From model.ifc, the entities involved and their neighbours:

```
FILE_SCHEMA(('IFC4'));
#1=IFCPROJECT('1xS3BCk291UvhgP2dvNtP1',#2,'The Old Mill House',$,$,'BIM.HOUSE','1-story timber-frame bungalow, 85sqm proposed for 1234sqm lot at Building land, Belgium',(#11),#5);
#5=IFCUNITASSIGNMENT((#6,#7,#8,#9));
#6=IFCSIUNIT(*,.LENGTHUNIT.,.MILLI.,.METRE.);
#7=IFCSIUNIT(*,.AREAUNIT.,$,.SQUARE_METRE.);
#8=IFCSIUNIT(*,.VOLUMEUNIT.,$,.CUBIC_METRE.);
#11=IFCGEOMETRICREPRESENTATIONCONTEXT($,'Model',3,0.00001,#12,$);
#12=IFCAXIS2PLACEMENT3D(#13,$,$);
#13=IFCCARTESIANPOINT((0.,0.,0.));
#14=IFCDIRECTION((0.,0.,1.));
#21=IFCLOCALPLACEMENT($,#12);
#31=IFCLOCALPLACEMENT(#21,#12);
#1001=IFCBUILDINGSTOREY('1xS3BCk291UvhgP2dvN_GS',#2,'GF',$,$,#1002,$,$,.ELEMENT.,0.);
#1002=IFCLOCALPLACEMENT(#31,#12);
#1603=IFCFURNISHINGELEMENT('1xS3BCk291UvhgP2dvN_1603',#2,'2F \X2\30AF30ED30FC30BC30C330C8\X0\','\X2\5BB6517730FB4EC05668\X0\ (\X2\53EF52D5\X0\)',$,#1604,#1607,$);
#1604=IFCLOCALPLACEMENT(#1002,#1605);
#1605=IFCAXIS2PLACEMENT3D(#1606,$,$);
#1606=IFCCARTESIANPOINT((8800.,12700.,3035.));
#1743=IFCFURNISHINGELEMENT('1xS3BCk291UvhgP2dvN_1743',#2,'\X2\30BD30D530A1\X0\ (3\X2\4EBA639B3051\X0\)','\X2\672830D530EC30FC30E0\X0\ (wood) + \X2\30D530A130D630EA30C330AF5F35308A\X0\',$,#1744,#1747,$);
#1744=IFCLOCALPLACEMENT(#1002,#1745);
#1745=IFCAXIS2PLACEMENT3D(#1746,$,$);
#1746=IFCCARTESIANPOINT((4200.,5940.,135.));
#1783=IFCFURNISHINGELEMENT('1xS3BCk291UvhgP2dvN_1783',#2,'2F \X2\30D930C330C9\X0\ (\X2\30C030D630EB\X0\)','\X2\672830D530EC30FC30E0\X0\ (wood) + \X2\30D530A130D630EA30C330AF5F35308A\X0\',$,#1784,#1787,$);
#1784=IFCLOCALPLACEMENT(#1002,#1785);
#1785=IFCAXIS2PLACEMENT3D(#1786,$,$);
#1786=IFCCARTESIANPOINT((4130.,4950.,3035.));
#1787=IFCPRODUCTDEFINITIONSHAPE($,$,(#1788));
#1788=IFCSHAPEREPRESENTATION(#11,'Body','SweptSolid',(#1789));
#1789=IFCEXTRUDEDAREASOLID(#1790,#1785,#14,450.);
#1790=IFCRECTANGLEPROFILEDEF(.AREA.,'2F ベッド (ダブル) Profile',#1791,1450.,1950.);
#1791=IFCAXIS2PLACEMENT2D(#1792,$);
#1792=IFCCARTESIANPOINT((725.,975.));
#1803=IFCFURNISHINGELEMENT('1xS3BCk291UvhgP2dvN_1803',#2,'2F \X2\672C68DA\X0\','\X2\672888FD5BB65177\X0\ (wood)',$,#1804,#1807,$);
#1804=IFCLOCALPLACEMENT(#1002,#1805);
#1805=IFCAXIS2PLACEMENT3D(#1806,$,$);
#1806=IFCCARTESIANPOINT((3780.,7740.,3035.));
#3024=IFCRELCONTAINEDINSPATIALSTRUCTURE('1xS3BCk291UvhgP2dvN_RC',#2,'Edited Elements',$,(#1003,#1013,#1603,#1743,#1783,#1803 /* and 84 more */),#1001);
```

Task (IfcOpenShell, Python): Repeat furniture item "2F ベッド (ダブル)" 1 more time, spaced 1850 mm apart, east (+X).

```python
import numpy as np
import ifcopenshell
import ifcopenshell.api.geometry
import ifcopenshell.api.root
import ifcopenshell.util.element
import ifcopenshell.util.placement
import ifcopenshell.util.unit

model = ifcopenshell.open("model.ifc")
unit_scale = ifcopenshell.util.unit.calculate_unit_scale(model)


def reuse_history(source, copy):
    """copy_class also copies each property set's owner history, people and application; keep the originals."""
    for rel in copy.IsDefinedBy:
        if rel.is_a("IfcRelDefinesByProperties") and (history := rel.RelatingPropertyDefinition.OwnerHistory):
            rel.RelatingPropertyDefinition.OwnerHistory = source.OwnerHistory
            ifcopenshell.util.element.remove_deep2(model, history)


source = model.by_id(1783)
base = ifcopenshell.util.placement.get_local_placement(source.ObjectPlacement)
step = np.array([1.0, 0.0, 0.0]) * 1.85 / unit_scale

for i in range(1, 2):
    copy = ifcopenshell.api.root.copy_class(model, product=source)
    copy.Representation = ifcopenshell.util.element.copy_deep(
        model, source.Representation, exclude=["IfcGeometricRepresentationContext", "IfcRepresentationMap"]
    )
    reuse_history(source, copy)
    matrix = base.copy()
    matrix[:3, 3] += i * step
    print("added at", matrix[:3, 3].round(3) + 0.0)
    ifcopenshell.api.geometry.edit_object_placement(model, product=copy, matrix=matrix, is_si=False)

model.write("model_v2.ifc")
```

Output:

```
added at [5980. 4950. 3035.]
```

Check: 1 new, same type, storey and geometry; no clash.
